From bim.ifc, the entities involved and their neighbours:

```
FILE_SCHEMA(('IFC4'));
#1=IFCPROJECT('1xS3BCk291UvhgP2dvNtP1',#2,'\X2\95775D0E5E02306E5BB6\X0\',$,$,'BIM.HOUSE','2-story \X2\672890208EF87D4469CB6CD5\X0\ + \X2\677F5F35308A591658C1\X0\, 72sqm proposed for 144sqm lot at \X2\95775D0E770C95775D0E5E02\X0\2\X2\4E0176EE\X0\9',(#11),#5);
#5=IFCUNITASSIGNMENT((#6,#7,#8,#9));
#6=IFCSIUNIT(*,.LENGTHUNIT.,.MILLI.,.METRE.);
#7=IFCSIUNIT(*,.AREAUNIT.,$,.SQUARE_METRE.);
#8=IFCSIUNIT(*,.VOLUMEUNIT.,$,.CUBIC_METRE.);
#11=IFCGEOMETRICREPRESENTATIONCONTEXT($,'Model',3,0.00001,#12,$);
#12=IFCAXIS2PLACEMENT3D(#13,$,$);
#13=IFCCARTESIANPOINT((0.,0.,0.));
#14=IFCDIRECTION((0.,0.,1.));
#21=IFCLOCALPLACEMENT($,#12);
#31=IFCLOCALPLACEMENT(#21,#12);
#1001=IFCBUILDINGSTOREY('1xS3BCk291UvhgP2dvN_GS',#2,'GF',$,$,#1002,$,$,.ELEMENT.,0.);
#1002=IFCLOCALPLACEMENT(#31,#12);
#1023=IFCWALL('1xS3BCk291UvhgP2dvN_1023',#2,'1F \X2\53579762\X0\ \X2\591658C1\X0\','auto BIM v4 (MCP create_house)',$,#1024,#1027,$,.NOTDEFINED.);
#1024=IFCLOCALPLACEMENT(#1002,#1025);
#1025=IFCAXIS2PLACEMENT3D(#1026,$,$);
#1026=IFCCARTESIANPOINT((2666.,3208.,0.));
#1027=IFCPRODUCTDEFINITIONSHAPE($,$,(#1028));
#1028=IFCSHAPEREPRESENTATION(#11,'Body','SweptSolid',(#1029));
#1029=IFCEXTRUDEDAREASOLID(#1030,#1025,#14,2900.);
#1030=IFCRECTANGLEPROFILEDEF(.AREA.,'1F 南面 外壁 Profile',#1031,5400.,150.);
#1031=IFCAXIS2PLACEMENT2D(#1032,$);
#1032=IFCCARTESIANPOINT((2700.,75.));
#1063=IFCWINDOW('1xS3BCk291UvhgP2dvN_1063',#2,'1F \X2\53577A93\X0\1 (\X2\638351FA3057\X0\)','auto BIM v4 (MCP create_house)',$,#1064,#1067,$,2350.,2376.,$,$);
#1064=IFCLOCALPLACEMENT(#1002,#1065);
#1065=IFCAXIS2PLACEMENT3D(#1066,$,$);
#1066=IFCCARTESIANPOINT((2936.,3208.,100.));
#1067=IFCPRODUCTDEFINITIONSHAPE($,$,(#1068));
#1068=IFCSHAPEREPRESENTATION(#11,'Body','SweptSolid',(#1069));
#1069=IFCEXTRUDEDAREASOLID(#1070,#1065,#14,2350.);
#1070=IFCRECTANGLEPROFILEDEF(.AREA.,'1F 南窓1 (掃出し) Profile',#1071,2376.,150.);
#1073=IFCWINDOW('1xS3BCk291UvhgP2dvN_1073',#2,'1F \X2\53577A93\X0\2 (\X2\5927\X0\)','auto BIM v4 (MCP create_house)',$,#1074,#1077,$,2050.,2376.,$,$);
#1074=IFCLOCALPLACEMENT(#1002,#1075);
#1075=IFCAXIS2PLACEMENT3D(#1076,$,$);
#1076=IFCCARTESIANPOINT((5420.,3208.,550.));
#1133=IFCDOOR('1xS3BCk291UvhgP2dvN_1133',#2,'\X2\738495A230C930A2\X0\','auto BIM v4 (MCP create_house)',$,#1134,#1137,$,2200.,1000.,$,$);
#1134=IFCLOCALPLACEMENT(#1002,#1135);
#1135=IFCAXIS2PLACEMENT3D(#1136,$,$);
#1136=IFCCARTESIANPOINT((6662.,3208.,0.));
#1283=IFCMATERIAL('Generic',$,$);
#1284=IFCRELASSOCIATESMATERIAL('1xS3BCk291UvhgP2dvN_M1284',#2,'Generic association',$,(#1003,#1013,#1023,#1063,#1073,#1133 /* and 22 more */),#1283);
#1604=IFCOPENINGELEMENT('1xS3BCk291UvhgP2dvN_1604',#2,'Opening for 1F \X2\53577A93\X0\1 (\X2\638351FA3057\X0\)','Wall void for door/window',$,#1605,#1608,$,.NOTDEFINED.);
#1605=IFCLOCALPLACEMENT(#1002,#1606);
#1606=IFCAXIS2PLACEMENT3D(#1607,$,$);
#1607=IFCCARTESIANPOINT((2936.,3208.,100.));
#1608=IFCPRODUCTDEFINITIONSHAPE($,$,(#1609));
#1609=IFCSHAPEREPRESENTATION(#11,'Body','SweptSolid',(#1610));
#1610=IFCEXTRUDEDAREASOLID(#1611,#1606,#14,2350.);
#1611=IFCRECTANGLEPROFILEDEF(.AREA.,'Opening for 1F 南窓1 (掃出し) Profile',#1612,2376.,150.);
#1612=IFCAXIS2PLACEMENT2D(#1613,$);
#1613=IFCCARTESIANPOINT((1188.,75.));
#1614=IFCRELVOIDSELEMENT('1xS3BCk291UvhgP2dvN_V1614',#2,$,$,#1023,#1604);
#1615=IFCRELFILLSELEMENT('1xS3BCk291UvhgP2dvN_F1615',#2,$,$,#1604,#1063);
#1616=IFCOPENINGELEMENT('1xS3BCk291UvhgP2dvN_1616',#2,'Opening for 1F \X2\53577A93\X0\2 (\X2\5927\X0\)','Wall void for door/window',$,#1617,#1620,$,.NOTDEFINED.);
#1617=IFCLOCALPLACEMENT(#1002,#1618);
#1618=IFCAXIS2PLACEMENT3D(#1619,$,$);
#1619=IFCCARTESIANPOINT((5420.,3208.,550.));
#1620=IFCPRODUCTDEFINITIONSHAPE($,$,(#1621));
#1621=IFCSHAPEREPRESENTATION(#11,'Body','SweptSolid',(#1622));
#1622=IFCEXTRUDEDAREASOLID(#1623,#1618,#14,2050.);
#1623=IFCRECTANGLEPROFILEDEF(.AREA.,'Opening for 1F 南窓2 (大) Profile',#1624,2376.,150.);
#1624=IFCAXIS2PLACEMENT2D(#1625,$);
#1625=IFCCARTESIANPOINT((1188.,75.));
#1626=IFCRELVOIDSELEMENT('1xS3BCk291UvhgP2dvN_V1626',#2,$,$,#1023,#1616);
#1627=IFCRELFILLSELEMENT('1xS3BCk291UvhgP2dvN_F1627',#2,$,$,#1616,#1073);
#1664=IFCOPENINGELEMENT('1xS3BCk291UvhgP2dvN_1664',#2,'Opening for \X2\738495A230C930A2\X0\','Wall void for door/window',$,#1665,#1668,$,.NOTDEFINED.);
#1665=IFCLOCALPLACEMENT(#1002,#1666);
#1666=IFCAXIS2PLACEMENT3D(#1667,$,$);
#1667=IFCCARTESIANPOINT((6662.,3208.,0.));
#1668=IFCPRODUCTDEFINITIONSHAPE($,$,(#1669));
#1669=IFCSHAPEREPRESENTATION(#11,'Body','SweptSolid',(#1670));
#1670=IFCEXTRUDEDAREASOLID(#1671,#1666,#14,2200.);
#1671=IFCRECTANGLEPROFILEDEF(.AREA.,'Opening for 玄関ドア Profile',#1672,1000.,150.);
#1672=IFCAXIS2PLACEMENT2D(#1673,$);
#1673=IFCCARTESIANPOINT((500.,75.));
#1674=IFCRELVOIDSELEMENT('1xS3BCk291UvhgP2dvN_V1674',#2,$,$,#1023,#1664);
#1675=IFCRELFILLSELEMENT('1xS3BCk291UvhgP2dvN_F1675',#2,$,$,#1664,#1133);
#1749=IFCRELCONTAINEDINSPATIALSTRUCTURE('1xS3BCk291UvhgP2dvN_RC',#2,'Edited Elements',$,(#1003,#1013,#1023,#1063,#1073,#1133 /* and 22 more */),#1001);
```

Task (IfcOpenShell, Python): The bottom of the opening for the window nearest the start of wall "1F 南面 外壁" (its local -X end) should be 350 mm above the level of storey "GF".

```python
import numpy as np
import ifcopenshell
import ifcopenshell.api.geometry
import ifcopenshell.geom
import ifcopenshell.util.element
import ifcopenshell.util.placement
import ifcopenshell.util.shape
import ifcopenshell.util.unit

model = ifcopenshell.open("bim.ifc")
unit_scale = ifcopenshell.util.unit.calculate_unit_scale(model)

window = model.by_guid("1xS3BCk291UvhgP2dvN_1063")
opening = window.FillsVoids[0].RelatingOpeningElement
storey = ifcopenshell.util.element.get_container(window, ifc_class="IfcBuildingStorey")
level = ifcopenshell.util.placement.get_local_placement(storey.ObjectPlacement)[2, 3]

# The opening's origin need not be at the sill, so measure its lowest point.
shape = ifcopenshell.geom.create_shape(ifcopenshell.geom.settings(), opening)
bottom = ifcopenshell.util.shape.get_shape_bottom_elevation(shape, shape.geometry) / unit_scale
dz = level + 350.0 - bottom

shift = np.array([0.0, 0.0, dz])
# The window is not placed relative to its opening, so move both.
for product in (opening, window):
    matrix = ifcopenshell.util.placement.get_local_placement(product.ObjectPlacement)
    matrix[:3, 3] += shift
    ifcopenshell.api.geometry.edit_object_placement(model, product=product, matrix=matrix, is_si=False)

print(f"moved by {dz * unit_scale:+.3f} m")

model.write("bim_updated.ifc")
```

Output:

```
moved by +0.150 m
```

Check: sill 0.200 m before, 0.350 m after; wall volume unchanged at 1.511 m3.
